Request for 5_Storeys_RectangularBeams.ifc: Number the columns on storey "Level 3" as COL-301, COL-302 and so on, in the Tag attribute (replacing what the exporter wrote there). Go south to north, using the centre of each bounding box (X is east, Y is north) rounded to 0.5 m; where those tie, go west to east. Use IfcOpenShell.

First a look at what the model holds.

```python
import ifcopenshell
import ifcopenshell.util.element
import ifcopenshell.util.placement

model = ifcopenshell.open("5_Storeys_RectangularBeams.ifc")
print(model.schema)
storey = next(s for s in model.by_type("IfcBuildingStorey") if s.Name == "Level 3")
columns = [e for e in ifcopenshell.util.element.get_decomposition(storey) if e.is_a("IfcColumn")]
for e in sorted(columns, key=lambda e: e.id()):
    origin = ifcopenshell.util.placement.get_local_placement(e.ObjectPlacement)[:3, 3]
    print(e.id(), e.Tag, e.Name, origin.round(2) + 0.0, sep=" | ")
```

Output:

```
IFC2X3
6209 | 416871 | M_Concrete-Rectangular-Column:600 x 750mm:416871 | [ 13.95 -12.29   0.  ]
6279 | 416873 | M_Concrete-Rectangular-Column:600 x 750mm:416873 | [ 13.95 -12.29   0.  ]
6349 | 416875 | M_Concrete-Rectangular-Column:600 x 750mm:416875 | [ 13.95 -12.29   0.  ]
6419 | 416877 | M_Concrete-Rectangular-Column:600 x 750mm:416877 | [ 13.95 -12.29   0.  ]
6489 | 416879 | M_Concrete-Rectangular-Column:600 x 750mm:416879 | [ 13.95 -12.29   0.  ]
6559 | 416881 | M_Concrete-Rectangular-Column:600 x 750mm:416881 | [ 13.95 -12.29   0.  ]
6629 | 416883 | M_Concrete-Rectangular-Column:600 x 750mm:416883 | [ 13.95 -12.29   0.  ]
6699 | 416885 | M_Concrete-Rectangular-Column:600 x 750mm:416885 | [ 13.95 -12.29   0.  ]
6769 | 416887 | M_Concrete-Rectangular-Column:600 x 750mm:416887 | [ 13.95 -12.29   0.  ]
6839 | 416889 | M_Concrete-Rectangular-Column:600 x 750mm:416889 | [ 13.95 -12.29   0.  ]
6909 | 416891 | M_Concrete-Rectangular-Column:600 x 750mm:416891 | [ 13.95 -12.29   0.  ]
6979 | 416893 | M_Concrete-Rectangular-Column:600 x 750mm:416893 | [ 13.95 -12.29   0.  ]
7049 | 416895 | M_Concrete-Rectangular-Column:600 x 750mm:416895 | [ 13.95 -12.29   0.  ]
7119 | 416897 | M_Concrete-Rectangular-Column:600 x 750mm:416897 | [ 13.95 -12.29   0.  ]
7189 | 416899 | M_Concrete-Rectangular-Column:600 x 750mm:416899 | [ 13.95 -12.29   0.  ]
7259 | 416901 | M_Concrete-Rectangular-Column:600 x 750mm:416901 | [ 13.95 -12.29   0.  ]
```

```python
import ifcopenshell
import ifcopenshell.geom
import ifcopenshell.util.element
import ifcopenshell.util.shape

model = ifcopenshell.open("5_Storeys_RectangularBeams.ifc")
settings = ifcopenshell.geom.settings()
settings.set("use-world-coords", True)


def centre(element):
    shape = ifcopenshell.geom.create_shape(settings, element)
    return ifcopenshell.util.shape.get_bbox_centroid(shape.geometry)


storey = next(s for s in model.by_type("IfcBuildingStorey") if s.Name == "Level 3")
columns = [e for e in ifcopenshell.util.element.get_decomposition(storey) if e.is_a("IfcColumn")]

# Insertion points can sit at a corner or the storey origin, so sort by the geometry (in metres).
centres = {e: centre(e) for e in columns}
columns.sort(key=lambda e: (round(centres[e][1] / 0.5), centres[e][0]))

for i, e in enumerate(columns, start=1):
    number = f"COL-3{i:02d}"
    e.Tag = number
    print(e.id(), number)

model.write("5_Storeys_RectangularBeams_updated.ifc")
```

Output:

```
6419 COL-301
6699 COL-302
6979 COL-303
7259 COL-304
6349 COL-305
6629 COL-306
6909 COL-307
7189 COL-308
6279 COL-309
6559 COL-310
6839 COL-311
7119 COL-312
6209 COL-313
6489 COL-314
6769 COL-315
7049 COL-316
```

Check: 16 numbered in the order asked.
